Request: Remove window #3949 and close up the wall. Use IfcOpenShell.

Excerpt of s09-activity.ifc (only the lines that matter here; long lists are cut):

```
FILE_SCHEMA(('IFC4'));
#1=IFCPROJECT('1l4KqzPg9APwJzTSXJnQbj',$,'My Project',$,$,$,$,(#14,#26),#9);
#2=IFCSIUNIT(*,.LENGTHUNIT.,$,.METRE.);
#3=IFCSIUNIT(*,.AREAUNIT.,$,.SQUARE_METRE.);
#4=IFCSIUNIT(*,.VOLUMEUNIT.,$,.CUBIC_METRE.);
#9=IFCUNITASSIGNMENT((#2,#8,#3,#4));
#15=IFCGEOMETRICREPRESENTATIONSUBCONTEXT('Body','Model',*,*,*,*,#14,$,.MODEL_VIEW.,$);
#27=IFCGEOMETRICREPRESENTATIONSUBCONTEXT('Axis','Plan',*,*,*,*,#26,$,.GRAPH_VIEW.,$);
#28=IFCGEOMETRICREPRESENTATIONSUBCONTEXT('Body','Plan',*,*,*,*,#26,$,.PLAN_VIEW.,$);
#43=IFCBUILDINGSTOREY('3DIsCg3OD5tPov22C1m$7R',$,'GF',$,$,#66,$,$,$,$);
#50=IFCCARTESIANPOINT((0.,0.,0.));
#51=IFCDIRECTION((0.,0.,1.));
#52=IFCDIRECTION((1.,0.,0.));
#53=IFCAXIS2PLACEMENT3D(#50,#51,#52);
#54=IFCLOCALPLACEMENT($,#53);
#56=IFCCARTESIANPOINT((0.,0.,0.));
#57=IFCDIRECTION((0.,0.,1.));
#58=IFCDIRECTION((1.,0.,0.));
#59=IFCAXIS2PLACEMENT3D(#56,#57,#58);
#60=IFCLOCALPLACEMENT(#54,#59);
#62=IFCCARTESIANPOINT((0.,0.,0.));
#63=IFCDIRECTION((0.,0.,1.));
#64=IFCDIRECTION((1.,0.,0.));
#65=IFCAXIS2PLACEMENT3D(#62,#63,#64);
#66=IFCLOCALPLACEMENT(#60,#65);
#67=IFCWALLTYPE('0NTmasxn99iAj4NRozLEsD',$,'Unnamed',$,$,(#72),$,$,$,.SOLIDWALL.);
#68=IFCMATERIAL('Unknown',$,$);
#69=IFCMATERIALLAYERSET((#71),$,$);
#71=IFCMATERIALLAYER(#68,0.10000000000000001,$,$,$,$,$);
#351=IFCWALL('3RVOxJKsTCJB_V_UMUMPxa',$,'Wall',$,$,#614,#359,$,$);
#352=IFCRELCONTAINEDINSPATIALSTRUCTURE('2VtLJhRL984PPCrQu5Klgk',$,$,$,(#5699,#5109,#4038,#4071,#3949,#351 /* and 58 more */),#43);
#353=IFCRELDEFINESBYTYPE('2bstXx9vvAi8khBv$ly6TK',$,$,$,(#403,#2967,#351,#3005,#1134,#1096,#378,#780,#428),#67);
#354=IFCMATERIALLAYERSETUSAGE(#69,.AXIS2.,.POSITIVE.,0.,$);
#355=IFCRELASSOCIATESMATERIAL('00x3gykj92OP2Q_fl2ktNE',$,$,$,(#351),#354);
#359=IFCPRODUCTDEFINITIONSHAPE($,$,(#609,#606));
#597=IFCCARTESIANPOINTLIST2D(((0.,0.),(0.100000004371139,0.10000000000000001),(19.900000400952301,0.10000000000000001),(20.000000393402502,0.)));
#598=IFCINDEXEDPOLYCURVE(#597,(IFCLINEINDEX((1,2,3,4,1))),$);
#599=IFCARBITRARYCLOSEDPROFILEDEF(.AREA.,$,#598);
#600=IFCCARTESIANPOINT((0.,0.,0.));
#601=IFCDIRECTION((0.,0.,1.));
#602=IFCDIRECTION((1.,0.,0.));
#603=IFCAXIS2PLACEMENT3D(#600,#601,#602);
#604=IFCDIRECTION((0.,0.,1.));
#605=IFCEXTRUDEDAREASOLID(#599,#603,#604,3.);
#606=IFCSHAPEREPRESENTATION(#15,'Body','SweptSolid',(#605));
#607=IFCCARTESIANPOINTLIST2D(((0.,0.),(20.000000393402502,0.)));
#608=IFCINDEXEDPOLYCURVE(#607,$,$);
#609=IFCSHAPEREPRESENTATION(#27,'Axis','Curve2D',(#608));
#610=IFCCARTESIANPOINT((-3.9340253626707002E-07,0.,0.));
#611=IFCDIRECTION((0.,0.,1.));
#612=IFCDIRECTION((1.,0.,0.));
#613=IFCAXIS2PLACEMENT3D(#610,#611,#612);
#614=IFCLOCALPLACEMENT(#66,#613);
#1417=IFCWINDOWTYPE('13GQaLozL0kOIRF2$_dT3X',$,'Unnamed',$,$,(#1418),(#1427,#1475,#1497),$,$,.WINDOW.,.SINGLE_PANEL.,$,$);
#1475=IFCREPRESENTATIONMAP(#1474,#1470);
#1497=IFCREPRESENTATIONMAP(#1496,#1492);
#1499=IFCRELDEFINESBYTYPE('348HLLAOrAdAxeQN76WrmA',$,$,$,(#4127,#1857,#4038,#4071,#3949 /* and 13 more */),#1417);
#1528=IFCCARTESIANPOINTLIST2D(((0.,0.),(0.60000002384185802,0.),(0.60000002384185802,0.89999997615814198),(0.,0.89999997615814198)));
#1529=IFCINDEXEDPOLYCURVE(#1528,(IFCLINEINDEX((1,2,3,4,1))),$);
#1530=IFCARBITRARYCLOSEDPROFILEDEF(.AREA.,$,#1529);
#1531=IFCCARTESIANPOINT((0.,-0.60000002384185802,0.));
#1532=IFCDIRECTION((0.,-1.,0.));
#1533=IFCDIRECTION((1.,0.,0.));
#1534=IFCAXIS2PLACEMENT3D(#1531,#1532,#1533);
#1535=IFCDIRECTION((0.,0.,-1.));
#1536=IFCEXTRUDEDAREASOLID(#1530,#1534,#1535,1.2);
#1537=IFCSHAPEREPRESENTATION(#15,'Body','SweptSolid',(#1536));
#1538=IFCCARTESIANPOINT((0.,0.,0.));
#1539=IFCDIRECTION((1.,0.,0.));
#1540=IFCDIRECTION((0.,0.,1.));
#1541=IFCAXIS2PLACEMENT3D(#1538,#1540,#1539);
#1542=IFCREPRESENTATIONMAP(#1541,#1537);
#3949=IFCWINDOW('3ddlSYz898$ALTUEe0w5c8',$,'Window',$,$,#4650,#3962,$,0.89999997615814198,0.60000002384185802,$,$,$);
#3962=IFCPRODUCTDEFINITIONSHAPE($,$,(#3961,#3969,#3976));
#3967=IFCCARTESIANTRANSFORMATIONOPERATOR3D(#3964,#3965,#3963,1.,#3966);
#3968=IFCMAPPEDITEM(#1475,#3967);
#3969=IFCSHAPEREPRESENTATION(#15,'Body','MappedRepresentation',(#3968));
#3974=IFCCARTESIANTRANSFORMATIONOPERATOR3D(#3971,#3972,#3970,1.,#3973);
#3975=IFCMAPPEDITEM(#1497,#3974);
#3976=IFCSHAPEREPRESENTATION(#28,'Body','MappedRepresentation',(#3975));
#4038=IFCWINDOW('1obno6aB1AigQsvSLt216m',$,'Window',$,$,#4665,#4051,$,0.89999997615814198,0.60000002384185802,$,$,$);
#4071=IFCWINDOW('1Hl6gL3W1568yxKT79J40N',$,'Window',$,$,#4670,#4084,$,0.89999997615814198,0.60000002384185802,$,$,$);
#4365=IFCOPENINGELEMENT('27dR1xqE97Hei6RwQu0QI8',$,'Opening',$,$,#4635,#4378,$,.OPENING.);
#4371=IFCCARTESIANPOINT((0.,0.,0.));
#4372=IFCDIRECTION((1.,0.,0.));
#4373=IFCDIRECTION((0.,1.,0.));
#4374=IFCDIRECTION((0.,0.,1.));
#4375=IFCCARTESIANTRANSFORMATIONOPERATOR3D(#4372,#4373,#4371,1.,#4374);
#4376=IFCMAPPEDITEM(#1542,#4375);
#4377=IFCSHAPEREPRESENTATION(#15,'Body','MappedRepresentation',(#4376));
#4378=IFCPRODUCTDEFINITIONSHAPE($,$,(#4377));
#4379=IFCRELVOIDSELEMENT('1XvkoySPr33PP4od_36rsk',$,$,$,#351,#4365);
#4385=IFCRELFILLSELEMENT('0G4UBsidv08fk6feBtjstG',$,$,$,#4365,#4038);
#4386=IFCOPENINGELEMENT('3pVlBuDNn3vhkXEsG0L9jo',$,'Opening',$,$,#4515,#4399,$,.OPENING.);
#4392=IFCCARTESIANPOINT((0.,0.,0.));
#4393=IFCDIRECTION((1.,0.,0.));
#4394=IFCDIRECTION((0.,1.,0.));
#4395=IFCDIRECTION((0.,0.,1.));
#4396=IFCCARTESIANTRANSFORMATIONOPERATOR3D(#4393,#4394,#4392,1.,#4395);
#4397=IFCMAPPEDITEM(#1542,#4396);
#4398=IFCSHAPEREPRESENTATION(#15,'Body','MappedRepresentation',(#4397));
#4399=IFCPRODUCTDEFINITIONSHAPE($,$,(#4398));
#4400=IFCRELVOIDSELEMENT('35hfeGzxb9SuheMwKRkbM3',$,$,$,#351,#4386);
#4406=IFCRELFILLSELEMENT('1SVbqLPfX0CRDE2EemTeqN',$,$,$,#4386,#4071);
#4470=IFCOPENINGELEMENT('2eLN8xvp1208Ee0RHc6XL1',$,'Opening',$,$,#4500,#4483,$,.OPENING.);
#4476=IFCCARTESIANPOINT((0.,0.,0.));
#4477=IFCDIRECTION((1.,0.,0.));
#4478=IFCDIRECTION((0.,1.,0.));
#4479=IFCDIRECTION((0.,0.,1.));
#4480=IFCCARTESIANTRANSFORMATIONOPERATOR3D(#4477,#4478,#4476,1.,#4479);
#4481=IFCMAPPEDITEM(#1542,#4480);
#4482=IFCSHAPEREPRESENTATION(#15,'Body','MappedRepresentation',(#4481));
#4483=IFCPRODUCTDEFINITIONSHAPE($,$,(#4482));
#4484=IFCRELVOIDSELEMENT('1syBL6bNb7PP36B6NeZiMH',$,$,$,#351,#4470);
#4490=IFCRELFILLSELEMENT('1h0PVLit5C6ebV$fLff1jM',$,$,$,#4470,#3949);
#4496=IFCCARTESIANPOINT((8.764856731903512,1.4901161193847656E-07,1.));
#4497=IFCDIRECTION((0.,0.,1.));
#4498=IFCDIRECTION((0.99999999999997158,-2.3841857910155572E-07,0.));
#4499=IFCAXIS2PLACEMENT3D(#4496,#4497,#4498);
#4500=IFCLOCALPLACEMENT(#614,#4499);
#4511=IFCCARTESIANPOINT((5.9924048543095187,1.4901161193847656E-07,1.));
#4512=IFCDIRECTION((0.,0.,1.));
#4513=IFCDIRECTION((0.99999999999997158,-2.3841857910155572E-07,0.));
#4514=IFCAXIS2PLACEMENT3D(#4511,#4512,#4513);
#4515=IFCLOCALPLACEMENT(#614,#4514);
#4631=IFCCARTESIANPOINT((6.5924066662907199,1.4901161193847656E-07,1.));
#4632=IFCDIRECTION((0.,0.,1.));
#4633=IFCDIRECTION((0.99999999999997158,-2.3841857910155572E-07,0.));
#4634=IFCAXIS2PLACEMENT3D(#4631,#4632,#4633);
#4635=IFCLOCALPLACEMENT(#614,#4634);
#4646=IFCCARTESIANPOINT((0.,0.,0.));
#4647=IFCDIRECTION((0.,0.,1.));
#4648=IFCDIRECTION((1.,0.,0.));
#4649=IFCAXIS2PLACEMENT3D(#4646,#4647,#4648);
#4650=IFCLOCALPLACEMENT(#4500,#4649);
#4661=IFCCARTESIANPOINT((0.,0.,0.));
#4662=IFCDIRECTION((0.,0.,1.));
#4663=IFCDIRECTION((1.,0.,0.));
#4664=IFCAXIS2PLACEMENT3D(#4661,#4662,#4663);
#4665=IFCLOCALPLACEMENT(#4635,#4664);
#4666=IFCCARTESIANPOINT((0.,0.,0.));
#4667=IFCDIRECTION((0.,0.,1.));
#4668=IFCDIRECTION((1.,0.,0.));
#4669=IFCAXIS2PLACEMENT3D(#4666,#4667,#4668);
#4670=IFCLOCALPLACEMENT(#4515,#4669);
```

```python
import ifcopenshell
import ifcopenshell.api.feature
import ifcopenshell.api.root
import ifcopenshell.geom
import ifcopenshell.util.shape

model = ifcopenshell.open("s09-activity.ifc")
settings = ifcopenshell.geom.settings()


def volume(element):
    """Net volume in cubic metres, openings subtracted."""
    shape = ifcopenshell.geom.create_shape(settings, element)
    return ifcopenshell.util.shape.get_volume(shape.geometry)


window = model.by_guid("3ddlSYz898$ALTUEe0w5c8")
opening = window.FillsVoids[0].RelatingOpeningElement
wall = opening.VoidsElements[0].RelatingBuildingElement
before = volume(wall)

ifcopenshell.api.root.remove_product(model, product=window)
ifcopenshell.api.feature.remove_feature(model, feature=opening)

after = volume(wall)

print(f"wall volume {before:.3f} -> {after:.3f} m3")

model.write("s09-activity_updated.ifc")
```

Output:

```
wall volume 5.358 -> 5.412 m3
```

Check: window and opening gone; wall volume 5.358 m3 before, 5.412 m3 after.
